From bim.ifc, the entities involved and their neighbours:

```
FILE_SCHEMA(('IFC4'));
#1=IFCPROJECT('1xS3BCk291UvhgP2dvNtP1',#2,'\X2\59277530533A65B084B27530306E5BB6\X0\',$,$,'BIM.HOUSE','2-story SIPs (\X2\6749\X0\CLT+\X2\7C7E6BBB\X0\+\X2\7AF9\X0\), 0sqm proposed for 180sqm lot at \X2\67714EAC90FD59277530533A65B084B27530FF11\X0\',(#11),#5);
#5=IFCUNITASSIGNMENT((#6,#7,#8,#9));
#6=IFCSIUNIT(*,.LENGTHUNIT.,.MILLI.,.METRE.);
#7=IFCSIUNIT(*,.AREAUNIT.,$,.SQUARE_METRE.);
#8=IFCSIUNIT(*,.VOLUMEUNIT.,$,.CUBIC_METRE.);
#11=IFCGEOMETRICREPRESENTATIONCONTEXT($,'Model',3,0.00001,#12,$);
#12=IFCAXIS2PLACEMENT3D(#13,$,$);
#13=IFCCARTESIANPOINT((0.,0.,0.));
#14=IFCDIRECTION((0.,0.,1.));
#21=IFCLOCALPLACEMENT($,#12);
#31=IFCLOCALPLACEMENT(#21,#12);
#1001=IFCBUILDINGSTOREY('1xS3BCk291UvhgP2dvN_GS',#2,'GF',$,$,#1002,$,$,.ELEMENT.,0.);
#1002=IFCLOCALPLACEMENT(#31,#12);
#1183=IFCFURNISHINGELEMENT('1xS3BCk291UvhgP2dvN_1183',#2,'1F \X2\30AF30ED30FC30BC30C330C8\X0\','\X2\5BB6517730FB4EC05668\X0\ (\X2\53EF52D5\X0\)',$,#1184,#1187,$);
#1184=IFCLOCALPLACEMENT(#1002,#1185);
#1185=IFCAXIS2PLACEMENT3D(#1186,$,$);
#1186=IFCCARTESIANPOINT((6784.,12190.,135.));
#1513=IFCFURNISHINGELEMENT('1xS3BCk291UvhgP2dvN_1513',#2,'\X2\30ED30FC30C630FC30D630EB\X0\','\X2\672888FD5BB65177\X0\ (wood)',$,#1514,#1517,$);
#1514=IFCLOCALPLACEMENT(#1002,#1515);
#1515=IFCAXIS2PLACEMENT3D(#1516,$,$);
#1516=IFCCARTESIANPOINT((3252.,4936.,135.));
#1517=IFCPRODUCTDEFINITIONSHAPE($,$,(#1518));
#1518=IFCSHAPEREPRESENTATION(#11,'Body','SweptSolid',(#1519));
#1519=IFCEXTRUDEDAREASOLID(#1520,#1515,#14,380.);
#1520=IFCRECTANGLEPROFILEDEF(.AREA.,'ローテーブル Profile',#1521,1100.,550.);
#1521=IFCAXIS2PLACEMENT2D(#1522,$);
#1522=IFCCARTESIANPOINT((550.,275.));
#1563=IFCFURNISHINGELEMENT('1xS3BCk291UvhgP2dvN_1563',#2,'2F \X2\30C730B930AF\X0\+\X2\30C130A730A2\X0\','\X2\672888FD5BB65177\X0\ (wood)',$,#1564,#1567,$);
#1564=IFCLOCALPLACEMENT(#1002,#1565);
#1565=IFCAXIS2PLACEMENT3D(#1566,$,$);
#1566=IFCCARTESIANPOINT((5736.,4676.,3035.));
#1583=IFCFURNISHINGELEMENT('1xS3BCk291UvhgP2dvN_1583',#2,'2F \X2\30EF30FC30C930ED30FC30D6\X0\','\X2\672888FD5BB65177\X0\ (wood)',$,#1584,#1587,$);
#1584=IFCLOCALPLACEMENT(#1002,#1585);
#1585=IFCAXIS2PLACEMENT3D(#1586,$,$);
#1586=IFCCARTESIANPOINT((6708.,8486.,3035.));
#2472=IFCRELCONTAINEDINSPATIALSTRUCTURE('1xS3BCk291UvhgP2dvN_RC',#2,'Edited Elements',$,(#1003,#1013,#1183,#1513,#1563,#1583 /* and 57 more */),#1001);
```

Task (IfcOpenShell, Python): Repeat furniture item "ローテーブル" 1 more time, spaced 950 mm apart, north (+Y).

```python
import numpy as np
import ifcopenshell
import ifcopenshell.api.geometry
import ifcopenshell.api.root
import ifcopenshell.util.element
import ifcopenshell.util.placement

model = ifcopenshell.open("bim.ifc")


def reuse_history(source, copy):
    """copy_class also copies each property set's owner history, people and application; keep the originals."""
    for rel in copy.IsDefinedBy:
        if rel.is_a("IfcRelDefinesByProperties") and (history := rel.RelatingPropertyDefinition.OwnerHistory):
            rel.RelatingPropertyDefinition.OwnerHistory = source.OwnerHistory
            ifcopenshell.util.element.remove_deep2(model, history)


source = model.by_guid("1xS3BCk291UvhgP2dvN_1513")
base = ifcopenshell.util.placement.get_local_placement(source.ObjectPlacement)
step = np.array([0.0, 1.0, 0.0]) * 950.0

for i in range(1, 2):
    copy = ifcopenshell.api.root.copy_class(model, product=source)
    copy.Representation = ifcopenshell.util.element.copy_deep(
        model, source.Representation, exclude=["IfcGeometricRepresentationContext", "IfcRepresentationMap"]
    )
    reuse_history(source, copy)
    matrix = base.copy()
    matrix[:3, 3] += i * step
    print("added at", matrix[:3, 3].round(3) + 0.0)
    ifcopenshell.api.geometry.edit_object_placement(model, product=copy, matrix=matrix, is_si=False)

model.write("bim_updated.ifc")
```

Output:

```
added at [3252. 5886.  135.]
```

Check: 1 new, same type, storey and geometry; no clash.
